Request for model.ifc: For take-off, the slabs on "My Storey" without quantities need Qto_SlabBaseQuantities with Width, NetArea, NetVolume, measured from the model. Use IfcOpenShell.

First a look at what the model holds.

```python
import ifcopenshell
import ifcopenshell.util.element
import ifcopenshell.util.unit

model = ifcopenshell.open("model.ifc")
print(model.schema)
for unit_type in ("LENGTHUNIT", "AREAUNIT", "VOLUMEUNIT"):
    print(unit_type, ifcopenshell.util.unit.calculate_unit_scale(model, unit_type))
storey = next(s for s in model.by_type("IfcBuildingStorey") if s.Name == "My Storey")
slabs = [e for e in ifcopenshell.util.element.get_decomposition(storey) if e.is_a("IfcSlab")]
for e in sorted(slabs, key=lambda e: e.id()):
    print(e.id(), e.is_a(), e.Name, list(ifcopenshell.util.element.get_psets(e, qtos_only=True)), sep=" | ")
```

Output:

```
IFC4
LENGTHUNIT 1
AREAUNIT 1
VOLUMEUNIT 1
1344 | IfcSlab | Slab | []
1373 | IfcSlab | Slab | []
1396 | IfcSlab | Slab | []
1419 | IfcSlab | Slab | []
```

```python
import ifcopenshell
import ifcopenshell.api.pset
import ifcopenshell.geom
import ifcopenshell.util.element
import ifcopenshell.util.shape
import ifcopenshell.util.unit

model = ifcopenshell.open("model.ifc")
unit_scale = ifcopenshell.util.unit.calculate_unit_scale(model)
area_scale = ifcopenshell.util.unit.calculate_unit_scale(model, "AREAUNIT")
volume_scale = ifcopenshell.util.unit.calculate_unit_scale(model, "VOLUMEUNIT")
settings = ifcopenshell.geom.settings()

storey = next(s for s in model.by_type("IfcBuildingStorey") if s.Name == "My Storey")
slabs = [e for e in ifcopenshell.util.element.get_decomposition(storey) if e.is_a("IfcSlab")]

for e in sorted(slabs, key=lambda e: e.id()):
    if ifcopenshell.util.element.get_psets(e, qtos_only=True, should_inherit=False):
        continue
    # Geometry comes back in metres, in the element's own axes.
    shape = ifcopenshell.geom.create_shape(settings, e)
    values = {
        "Width": ifcopenshell.util.shape.get_z(shape.geometry) / unit_scale,
        "NetArea": ifcopenshell.util.shape.get_footprint_area(shape.geometry) / area_scale,
        "NetVolume": ifcopenshell.util.shape.get_volume(shape.geometry) / volume_scale,
    }
    qto = ifcopenshell.api.pset.add_qto(model, product=e, name="Qto_SlabBaseQuantities")
    ifcopenshell.api.pset.edit_qto(model, qto=qto, properties=values)
    print(e.id(), {k: round(v, 3) for k, v in values.items()})

model.write("model_edited.ifc")
```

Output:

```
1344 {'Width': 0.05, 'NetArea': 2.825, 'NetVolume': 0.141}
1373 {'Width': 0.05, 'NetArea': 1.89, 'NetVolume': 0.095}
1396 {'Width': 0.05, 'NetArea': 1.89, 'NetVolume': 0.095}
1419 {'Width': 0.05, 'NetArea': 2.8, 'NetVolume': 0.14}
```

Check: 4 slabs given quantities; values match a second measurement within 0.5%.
